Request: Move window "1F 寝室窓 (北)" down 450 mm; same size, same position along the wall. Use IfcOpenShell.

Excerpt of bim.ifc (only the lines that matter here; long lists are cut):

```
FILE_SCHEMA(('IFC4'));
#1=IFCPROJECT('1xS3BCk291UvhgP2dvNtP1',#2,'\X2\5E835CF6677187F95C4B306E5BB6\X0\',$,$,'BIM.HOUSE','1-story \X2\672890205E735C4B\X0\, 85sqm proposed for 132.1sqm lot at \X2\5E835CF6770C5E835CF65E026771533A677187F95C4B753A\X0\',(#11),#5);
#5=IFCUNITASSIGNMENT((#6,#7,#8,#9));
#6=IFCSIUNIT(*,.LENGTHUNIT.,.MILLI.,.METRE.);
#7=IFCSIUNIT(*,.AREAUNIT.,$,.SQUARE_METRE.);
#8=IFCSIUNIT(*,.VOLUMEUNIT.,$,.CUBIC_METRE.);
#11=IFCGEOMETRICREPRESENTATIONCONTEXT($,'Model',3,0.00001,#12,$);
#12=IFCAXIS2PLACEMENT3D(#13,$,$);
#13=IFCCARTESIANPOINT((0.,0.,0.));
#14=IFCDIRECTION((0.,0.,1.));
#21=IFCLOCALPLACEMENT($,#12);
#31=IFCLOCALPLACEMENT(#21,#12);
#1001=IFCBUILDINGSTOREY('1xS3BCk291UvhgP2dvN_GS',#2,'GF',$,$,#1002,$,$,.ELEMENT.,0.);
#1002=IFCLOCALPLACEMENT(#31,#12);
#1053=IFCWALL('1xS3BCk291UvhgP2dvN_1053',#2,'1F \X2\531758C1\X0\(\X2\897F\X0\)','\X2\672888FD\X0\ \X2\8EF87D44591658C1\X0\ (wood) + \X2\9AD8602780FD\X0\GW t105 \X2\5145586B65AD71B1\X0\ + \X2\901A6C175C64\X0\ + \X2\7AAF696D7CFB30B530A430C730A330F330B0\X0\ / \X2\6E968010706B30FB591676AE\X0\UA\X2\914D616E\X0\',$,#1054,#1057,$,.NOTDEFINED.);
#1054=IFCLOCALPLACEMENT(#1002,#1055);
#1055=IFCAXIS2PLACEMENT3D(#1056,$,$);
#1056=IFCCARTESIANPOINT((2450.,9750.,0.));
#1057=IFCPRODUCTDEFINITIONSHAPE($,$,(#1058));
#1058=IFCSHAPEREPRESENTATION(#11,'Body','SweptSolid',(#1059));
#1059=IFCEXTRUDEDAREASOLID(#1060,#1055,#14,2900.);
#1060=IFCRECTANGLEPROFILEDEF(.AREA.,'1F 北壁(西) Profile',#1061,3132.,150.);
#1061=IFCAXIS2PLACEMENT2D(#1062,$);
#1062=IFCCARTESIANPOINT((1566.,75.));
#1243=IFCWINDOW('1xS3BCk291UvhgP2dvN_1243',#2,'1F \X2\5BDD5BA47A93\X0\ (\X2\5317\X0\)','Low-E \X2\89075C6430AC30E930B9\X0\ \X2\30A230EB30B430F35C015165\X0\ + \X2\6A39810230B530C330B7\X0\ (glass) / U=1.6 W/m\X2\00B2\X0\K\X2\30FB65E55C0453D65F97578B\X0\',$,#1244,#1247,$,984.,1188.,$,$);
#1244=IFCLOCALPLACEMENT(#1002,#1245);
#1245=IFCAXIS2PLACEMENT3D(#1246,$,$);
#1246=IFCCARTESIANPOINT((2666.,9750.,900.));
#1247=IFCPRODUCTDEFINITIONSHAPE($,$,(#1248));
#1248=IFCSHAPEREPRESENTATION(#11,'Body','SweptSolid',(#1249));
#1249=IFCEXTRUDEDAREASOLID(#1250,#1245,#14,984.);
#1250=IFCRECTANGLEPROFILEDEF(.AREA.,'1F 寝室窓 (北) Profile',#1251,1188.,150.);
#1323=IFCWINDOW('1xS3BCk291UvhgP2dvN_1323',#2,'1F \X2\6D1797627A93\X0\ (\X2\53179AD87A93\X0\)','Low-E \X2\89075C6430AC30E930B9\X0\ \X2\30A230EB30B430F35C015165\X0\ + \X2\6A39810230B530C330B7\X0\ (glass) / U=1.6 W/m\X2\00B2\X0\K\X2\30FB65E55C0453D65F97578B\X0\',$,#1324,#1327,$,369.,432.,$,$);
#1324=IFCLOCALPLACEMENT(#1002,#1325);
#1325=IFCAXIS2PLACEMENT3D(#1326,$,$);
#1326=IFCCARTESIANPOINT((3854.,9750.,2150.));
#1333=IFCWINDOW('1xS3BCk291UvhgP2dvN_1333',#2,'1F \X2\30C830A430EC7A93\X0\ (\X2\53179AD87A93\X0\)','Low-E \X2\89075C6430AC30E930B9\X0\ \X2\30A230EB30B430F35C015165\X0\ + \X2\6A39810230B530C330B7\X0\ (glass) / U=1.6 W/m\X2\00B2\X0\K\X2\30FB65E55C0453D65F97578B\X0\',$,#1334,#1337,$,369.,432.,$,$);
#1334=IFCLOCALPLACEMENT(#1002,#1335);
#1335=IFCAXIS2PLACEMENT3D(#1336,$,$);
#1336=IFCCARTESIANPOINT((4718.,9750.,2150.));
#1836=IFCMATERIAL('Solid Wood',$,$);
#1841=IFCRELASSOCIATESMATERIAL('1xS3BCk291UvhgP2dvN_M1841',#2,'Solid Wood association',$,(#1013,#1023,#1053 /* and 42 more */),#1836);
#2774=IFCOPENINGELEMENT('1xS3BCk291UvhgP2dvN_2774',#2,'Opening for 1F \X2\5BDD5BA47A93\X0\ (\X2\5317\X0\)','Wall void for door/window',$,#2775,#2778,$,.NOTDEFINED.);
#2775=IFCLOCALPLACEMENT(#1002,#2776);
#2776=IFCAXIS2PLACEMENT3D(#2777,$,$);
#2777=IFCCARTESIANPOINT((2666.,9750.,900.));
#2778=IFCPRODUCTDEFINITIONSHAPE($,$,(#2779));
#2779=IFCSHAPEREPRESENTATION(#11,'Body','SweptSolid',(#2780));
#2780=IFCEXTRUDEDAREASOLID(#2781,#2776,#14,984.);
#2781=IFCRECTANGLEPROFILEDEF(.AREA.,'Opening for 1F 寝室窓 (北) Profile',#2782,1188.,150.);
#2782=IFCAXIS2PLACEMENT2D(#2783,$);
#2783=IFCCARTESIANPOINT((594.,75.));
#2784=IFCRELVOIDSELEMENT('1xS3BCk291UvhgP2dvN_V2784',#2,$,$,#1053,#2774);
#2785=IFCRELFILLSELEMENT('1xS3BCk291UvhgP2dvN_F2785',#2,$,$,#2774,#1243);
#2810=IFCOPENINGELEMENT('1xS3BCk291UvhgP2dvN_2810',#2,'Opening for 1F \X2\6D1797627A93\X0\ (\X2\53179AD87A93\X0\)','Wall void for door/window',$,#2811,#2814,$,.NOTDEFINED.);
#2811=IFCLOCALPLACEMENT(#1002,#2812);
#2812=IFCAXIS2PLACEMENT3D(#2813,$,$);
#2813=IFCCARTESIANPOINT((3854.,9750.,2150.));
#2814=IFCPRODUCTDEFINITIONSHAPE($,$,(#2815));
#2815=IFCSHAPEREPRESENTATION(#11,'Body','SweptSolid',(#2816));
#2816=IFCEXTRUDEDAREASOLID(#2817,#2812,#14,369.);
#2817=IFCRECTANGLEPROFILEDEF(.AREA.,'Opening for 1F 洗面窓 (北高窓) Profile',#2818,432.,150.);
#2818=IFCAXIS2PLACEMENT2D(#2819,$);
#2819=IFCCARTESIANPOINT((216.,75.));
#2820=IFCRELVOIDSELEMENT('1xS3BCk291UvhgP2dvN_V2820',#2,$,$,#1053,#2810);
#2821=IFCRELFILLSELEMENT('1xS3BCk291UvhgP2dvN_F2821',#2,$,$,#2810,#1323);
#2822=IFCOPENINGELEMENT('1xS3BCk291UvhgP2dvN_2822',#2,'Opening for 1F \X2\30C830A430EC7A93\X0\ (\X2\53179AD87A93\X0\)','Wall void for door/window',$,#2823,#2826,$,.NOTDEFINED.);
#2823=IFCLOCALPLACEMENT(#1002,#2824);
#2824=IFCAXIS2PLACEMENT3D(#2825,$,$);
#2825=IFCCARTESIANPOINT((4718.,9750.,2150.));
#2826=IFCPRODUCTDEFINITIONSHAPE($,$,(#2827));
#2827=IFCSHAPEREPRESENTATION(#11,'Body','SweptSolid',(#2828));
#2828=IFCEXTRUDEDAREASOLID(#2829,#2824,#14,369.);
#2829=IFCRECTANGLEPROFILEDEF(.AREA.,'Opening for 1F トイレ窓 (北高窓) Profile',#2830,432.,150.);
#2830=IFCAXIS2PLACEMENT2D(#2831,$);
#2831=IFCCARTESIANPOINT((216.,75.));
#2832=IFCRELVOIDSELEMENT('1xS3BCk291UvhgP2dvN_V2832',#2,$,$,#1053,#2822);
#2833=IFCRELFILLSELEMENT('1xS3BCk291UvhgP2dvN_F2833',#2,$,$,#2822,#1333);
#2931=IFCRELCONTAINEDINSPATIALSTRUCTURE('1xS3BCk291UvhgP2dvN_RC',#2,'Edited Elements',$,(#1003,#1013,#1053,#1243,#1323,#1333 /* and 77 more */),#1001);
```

```python
import numpy as np
import ifcopenshell
import ifcopenshell.api.geometry
import ifcopenshell.util.placement
import ifcopenshell.util.unit

model = ifcopenshell.open("bim.ifc")
unit_scale = ifcopenshell.util.unit.calculate_unit_scale(model)

window = model.by_guid("1xS3BCk291UvhgP2dvN_1243")
opening = window.FillsVoids[0].RelatingOpeningElement
dz = -0.45 / unit_scale

shift = np.array([0.0, 0.0, dz])
# The window is not placed relative to its opening, so move both.
for product in (opening, window):
    matrix = ifcopenshell.util.placement.get_local_placement(product.ObjectPlacement)
    matrix[:3, 3] += shift
    ifcopenshell.api.geometry.edit_object_placement(model, product=product, matrix=matrix, is_si=False)

print(f"moved by {dz * unit_scale:+.3f} m")

model.write("bim-out.ifc")
```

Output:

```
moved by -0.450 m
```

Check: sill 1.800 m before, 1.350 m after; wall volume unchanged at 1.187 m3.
